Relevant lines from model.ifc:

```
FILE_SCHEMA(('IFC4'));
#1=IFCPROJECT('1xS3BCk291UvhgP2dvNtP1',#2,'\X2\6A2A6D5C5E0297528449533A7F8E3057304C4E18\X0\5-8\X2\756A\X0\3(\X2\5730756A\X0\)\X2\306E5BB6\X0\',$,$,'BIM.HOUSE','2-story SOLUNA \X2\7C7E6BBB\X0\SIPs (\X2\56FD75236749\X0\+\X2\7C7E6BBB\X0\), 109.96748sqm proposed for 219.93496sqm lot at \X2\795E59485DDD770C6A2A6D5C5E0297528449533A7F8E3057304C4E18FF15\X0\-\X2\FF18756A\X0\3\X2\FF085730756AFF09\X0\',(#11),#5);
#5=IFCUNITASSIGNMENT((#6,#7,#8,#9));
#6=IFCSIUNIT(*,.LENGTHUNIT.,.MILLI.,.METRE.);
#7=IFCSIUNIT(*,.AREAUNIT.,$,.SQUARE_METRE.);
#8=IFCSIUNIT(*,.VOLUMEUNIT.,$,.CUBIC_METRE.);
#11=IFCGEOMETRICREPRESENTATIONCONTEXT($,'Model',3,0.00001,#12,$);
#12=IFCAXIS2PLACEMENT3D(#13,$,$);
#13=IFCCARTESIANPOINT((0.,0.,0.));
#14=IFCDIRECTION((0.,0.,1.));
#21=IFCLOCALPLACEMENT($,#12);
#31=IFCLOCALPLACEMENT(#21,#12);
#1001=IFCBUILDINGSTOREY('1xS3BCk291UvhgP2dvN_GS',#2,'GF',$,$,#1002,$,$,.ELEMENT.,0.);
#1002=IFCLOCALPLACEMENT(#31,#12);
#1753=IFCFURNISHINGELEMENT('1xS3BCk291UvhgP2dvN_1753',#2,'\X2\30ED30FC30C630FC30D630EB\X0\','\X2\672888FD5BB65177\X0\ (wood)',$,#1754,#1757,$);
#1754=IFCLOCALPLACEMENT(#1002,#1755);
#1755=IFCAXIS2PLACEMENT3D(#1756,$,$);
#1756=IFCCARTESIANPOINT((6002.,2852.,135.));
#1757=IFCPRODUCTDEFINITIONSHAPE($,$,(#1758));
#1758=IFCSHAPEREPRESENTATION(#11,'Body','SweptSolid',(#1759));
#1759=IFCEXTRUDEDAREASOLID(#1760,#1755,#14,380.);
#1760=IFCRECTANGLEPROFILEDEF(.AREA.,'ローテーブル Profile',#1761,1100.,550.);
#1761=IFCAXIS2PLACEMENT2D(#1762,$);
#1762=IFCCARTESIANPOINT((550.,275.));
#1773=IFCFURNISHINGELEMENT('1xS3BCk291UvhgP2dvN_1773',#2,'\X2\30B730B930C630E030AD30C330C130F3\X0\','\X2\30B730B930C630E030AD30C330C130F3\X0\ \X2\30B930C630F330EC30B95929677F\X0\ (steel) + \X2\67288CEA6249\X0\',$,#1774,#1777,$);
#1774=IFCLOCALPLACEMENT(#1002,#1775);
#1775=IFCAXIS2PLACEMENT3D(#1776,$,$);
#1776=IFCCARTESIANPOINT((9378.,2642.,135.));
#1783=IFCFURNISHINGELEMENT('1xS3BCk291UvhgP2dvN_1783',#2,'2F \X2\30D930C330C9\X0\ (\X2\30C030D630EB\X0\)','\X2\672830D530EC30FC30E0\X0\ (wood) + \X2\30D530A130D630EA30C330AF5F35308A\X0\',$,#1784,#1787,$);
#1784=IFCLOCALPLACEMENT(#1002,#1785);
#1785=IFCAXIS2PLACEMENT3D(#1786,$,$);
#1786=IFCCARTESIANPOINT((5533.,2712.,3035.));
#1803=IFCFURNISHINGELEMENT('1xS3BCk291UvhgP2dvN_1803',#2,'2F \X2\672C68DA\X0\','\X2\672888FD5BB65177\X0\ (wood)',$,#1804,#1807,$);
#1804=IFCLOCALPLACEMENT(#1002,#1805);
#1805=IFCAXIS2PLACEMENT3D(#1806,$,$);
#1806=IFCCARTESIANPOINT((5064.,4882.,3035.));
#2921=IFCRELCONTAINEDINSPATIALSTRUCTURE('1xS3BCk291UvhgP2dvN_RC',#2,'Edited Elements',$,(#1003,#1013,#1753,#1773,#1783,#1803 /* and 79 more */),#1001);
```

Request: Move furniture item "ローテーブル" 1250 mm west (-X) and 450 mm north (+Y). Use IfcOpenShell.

```python
import ifcopenshell
import ifcopenshell.api.geometry
import ifcopenshell.util.placement
import ifcopenshell.util.unit

model = ifcopenshell.open("model.ifc")
unit_scale = ifcopenshell.util.unit.calculate_unit_scale(model)

item = model.by_id(1753)
matrix = ifcopenshell.util.placement.get_local_placement(item.ObjectPlacement)
matrix[0, 3] -= 1.25 / unit_scale
matrix[1, 3] += 0.45 / unit_scale
ifcopenshell.api.geometry.edit_object_placement(model, product=item, matrix=matrix, is_si=False)

print(ifcopenshell.util.placement.get_local_placement(item.ObjectPlacement).round(3) + 0.0)

model.write("model_v2.ifc")
```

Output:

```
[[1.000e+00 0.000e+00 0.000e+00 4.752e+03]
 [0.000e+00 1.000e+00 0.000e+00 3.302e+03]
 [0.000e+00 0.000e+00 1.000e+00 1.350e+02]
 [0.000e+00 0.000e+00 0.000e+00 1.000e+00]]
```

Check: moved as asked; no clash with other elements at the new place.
